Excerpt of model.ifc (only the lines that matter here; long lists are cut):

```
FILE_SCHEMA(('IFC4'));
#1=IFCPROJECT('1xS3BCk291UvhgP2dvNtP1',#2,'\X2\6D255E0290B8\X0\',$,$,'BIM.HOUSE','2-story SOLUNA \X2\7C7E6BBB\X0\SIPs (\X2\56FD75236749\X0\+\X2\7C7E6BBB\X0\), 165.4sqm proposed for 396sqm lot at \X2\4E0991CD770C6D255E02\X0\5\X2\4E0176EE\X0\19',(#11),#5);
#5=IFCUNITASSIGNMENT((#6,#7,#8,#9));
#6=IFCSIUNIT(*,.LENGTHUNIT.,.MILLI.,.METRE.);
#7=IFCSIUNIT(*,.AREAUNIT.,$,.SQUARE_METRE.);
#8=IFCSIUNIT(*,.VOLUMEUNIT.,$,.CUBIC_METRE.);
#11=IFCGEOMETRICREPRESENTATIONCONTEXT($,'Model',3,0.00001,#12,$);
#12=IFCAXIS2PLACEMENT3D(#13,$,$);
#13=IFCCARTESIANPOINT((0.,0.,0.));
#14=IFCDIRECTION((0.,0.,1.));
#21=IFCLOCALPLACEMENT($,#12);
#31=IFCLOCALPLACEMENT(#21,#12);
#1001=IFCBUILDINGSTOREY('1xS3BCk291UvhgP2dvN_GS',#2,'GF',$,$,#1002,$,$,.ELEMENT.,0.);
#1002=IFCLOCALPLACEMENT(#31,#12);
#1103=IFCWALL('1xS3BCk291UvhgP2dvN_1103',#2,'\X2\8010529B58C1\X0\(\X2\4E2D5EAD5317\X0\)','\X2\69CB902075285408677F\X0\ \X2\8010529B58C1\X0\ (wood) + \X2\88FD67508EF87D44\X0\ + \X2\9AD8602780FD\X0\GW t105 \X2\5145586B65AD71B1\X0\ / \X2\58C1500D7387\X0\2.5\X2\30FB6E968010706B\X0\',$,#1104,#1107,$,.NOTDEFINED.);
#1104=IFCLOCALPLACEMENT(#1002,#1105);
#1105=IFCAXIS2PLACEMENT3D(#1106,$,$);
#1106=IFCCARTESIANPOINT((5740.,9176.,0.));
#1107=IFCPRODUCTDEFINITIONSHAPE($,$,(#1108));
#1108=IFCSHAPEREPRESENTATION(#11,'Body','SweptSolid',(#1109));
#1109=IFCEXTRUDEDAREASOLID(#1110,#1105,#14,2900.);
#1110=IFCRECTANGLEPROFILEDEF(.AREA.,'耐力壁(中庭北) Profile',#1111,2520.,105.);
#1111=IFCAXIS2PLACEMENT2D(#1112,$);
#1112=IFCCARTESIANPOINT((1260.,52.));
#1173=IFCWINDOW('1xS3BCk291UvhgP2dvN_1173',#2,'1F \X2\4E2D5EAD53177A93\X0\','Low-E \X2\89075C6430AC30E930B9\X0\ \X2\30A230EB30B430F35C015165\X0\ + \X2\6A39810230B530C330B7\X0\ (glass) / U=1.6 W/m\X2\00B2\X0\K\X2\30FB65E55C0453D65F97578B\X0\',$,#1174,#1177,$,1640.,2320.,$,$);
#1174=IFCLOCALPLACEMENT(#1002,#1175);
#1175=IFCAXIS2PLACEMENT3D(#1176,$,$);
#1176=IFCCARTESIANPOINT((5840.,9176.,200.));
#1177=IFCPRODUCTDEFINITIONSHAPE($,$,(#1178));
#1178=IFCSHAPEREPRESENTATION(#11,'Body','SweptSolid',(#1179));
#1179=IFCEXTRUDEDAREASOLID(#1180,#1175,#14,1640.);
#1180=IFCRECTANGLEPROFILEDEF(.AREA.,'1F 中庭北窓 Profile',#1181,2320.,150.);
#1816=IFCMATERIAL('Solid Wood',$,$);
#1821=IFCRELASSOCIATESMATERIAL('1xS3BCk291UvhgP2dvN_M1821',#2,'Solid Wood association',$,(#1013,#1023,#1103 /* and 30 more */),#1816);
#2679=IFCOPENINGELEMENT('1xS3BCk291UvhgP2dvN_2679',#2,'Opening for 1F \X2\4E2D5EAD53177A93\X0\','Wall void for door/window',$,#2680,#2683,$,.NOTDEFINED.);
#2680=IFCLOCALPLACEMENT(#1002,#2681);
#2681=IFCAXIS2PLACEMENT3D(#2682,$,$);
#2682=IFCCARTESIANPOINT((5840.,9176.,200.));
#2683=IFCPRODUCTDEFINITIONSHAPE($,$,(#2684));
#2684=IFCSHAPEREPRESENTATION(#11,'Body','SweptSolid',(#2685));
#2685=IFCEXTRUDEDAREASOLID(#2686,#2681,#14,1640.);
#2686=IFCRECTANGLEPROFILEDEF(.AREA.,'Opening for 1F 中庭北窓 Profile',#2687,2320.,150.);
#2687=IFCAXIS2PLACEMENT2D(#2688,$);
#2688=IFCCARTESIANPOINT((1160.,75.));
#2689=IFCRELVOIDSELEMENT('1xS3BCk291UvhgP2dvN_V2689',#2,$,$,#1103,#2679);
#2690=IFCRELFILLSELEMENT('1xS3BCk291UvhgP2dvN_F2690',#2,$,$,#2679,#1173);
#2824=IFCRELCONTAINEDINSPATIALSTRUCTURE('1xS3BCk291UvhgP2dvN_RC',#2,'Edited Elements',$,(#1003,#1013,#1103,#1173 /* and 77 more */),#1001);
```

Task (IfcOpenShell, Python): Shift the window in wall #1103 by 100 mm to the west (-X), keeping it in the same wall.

```python
import ifcopenshell
import ifcopenshell.api.geometry
import ifcopenshell.util.placement
import ifcopenshell.util.unit

model = ifcopenshell.open("model.ifc")
unit_scale = ifcopenshell.util.unit.calculate_unit_scale(model)

window = model.by_id(1173)
opening = window.FillsVoids[0].RelatingOpeningElement
wall = opening.VoidsElements[0].RelatingBuildingElement

wall_matrix = ifcopenshell.util.placement.get_local_placement(wall.ObjectPlacement)
shift = wall_matrix[:3, 0] * -0.1 / unit_scale
before = ifcopenshell.util.placement.get_local_placement(window.ObjectPlacement)[:3, 3].copy()

# The window is not placed relative to its opening, so move both.
for product in (opening, window):
    matrix = ifcopenshell.util.placement.get_local_placement(product.ObjectPlacement)
    matrix[:3, 3] += shift
    ifcopenshell.api.geometry.edit_object_placement(model, product=product, matrix=matrix, is_si=False)

after = ifcopenshell.util.placement.get_local_placement(window.ObjectPlacement)[:3, 3]
print("window moved by", (after - before).round(3) + 0.0)

model.write("model_updated.ifc")
```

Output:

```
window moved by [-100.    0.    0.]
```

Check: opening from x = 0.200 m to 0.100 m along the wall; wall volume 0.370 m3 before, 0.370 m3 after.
